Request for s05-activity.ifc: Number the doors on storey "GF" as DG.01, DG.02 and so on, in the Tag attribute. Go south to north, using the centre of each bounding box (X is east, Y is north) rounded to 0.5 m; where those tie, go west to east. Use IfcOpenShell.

First a look at what the model holds.

```python
import ifcopenshell
import ifcopenshell.util.element
import ifcopenshell.util.placement

model = ifcopenshell.open("s05-activity.ifc")
print(model.schema)
storey = next(s for s in model.by_type("IfcBuildingStorey") if s.Name == "GF")
doors = [e for e in ifcopenshell.util.element.get_decomposition(storey) if e.is_a("IfcDoor")]
for e in sorted(doors, key=lambda e: e.id()):
    origin = ifcopenshell.util.placement.get_local_placement(e.ObjectPlacement)[:3, 3]
    print(e.id(), e.Tag, e.Name, origin.round(2) + 0.0, sep=" | ")
```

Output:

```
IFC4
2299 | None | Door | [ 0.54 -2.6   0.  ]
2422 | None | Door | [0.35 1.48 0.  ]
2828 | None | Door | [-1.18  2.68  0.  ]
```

```python
import ifcopenshell
import ifcopenshell.geom
import ifcopenshell.util.element
import ifcopenshell.util.shape

model = ifcopenshell.open("s05-activity.ifc")
settings = ifcopenshell.geom.settings()
settings.set("use-world-coords", True)


def centre(element):
    shape = ifcopenshell.geom.create_shape(settings, element)
    return ifcopenshell.util.shape.get_bbox_centroid(shape.geometry)


storey = next(s for s in model.by_type("IfcBuildingStorey") if s.Name == "GF")
doors = [e for e in ifcopenshell.util.element.get_decomposition(storey) if e.is_a("IfcDoor")]

# Insertion points can sit at a corner or the storey origin, so sort by the geometry (in metres).
centres = {e: centre(e) for e in doors}
doors.sort(key=lambda e: (round(centres[e][1] / 0.5), centres[e][0]))

for i, e in enumerate(doors, start=1):
    number = f"DG.{i:02d}"
    e.Tag = number
    print(e.id(), number)

model.write("s05-activity-out.ifc")
```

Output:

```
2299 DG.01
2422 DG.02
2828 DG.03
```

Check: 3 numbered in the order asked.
